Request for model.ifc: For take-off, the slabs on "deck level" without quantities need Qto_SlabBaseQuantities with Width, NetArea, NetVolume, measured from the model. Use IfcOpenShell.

First a look at what the model holds.

```python
import ifcopenshell
import ifcopenshell.util.element
import ifcopenshell.util.unit

model = ifcopenshell.open("model.ifc")
print(model.schema)
for unit_type in ("LENGTHUNIT", "AREAUNIT", "VOLUMEUNIT"):
    print(unit_type, ifcopenshell.util.unit.calculate_unit_scale(model, unit_type))
storey = next(s for s in model.by_type("IfcBuildingStorey") if s.Name == "deck level")
slabs = [e for e in ifcopenshell.util.element.get_decomposition(storey) if e.is_a("IfcSlab")]
for e in sorted(slabs, key=lambda e: e.id()):
    print(e.id(), e.is_a(), e.Name, list(ifcopenshell.util.element.get_psets(e, qtos_only=True)), sep=" | ")
```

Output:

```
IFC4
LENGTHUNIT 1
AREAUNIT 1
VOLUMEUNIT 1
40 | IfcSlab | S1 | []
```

```python
import ifcopenshell
import ifcopenshell.api.pset
import ifcopenshell.geom
import ifcopenshell.util.element
import ifcopenshell.util.shape
import ifcopenshell.util.unit

model = ifcopenshell.open("model.ifc")
unit_scale = ifcopenshell.util.unit.calculate_unit_scale(model)
area_scale = ifcopenshell.util.unit.calculate_unit_scale(model, "AREAUNIT")
volume_scale = ifcopenshell.util.unit.calculate_unit_scale(model, "VOLUMEUNIT")
settings = ifcopenshell.geom.settings()

storey = next(s for s in model.by_type("IfcBuildingStorey") if s.Name == "deck level")
slabs = [e for e in ifcopenshell.util.element.get_decomposition(storey) if e.is_a("IfcSlab")]

for e in sorted(slabs, key=lambda e: e.id()):
    if ifcopenshell.util.element.get_psets(e, qtos_only=True, should_inherit=False):
        continue
    # Geometry comes back in metres, in the element's own axes.
    shape = ifcopenshell.geom.create_shape(settings, e)
    values = {
        "Width": ifcopenshell.util.shape.get_z(shape.geometry) / unit_scale,
        "NetArea": ifcopenshell.util.shape.get_footprint_area(shape.geometry) / area_scale,
        "NetVolume": ifcopenshell.util.shape.get_volume(shape.geometry) / volume_scale,
    }
    qto = ifcopenshell.api.pset.add_qto(model, product=e, name="Qto_SlabBaseQuantities")
    ifcopenshell.api.pset.edit_qto(model, qto=qto, properties=values)
    print(e.id(), {k: round(v, 3) for k, v in values.items()})

model.write("model_rev.ifc")
```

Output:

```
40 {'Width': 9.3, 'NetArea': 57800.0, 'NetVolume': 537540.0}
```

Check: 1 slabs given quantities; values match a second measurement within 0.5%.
